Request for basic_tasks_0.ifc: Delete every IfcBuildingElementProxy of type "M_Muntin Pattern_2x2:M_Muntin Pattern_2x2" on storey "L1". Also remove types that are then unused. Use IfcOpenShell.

First a look at what the model holds.

```python
import ifcopenshell
import ifcopenshell.util.element

model = ifcopenshell.open("basic_tasks_0.ifc")
print(model.schema)
storey = next(s for s in model.by_type("IfcBuildingStorey") if s.Name == "L1")
proxies = [e for e in ifcopenshell.util.element.get_decomposition(storey) if e.is_a("IfcBuildingElementProxy")]
seen = {}
for e in proxies:
    element_type = ifcopenshell.util.element.get_type(e)
    name = element_type.Name if element_type not in (None, e) else None
    seen[name] = seen.get(name, 0) + 1
for name, count in sorted(seen.items(), key=str):
    print(count, "x", name)
```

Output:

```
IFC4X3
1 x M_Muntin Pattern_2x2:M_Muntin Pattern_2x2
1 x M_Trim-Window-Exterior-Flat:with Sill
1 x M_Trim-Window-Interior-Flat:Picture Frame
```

```python
import ifcopenshell
import ifcopenshell.api.root
import ifcopenshell.util.element

model = ifcopenshell.open("basic_tasks_0.ifc")

storey = next(s for s in model.by_type("IfcBuildingStorey") if s.Name == "L1")
proxies = [e for e in ifcopenshell.util.element.get_decomposition(storey) if e.is_a("IfcBuildingElementProxy")]
targets = [e for e in proxies if (t := ifcopenshell.util.element.get_type(e)) not in (None, e) and t.Name == "M_Muntin Pattern_2x2:M_Muntin Pattern_2x2"]
types = {ifcopenshell.util.element.get_type(e) for e in targets} - {None, *targets}

for e in targets:
    ifcopenshell.api.root.remove_product(model, product=e)
print(len(targets), "removed")

unused = [t for t in types if not ifcopenshell.util.element.get_types(t)]
for t in unused:
    ifcopenshell.api.root.remove_product(model, product=t)
print(len(unused), "unused types removed")

model.write("basic_tasks_0_rev.ifc")
```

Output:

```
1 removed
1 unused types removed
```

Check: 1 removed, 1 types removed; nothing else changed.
